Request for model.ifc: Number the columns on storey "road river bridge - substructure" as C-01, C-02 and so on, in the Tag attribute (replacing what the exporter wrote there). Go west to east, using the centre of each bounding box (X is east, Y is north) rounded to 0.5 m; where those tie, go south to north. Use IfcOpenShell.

First a look at what the model holds.

```python
import ifcopenshell
import ifcopenshell.util.element
import ifcopenshell.util.placement

model = ifcopenshell.open("model.ifc")
print(model.schema)
storey = next(s for s in model.by_type("IfcBuildingStorey") if s.Name == "road river bridge - substructure")
columns = [e for e in ifcopenshell.util.element.get_decomposition(storey) if e.is_a("IfcColumn")]
for e in sorted(columns, key=lambda e: e.id()):
    origin = ifcopenshell.util.placement.get_local_placement(e.ObjectPlacement)[:3, 3]
    print(e.id(), e.Tag, e.Name, origin.round(2) + 0.0, sep=" | ")
```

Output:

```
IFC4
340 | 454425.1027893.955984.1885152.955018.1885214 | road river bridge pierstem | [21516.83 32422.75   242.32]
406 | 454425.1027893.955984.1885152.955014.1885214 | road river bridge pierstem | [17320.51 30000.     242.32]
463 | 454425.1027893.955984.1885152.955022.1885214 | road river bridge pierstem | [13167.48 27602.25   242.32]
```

```python
import ifcopenshell
import ifcopenshell.geom
import ifcopenshell.util.element
import ifcopenshell.util.shape

model = ifcopenshell.open("model.ifc")
settings = ifcopenshell.geom.settings()
settings.set("use-world-coords", True)


def centre(element):
    shape = ifcopenshell.geom.create_shape(settings, element)
    return ifcopenshell.util.shape.get_bbox_centroid(shape.geometry)


storey = next(s for s in model.by_type("IfcBuildingStorey") if s.Name == "road river bridge - substructure")
columns = [e for e in ifcopenshell.util.element.get_decomposition(storey) if e.is_a("IfcColumn")]

# Insertion points can sit at a corner or the storey origin, so sort by the geometry (in metres).
centres = {e: centre(e) for e in columns}
columns.sort(key=lambda e: (round(centres[e][0] / 0.5), centres[e][1]))

for i, e in enumerate(columns, start=1):
    number = f"C-{i:02d}"
    e.Tag = number
    print(e.id(), number)

model.write("model_updated.ifc")
```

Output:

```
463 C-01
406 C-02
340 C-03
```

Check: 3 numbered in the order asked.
